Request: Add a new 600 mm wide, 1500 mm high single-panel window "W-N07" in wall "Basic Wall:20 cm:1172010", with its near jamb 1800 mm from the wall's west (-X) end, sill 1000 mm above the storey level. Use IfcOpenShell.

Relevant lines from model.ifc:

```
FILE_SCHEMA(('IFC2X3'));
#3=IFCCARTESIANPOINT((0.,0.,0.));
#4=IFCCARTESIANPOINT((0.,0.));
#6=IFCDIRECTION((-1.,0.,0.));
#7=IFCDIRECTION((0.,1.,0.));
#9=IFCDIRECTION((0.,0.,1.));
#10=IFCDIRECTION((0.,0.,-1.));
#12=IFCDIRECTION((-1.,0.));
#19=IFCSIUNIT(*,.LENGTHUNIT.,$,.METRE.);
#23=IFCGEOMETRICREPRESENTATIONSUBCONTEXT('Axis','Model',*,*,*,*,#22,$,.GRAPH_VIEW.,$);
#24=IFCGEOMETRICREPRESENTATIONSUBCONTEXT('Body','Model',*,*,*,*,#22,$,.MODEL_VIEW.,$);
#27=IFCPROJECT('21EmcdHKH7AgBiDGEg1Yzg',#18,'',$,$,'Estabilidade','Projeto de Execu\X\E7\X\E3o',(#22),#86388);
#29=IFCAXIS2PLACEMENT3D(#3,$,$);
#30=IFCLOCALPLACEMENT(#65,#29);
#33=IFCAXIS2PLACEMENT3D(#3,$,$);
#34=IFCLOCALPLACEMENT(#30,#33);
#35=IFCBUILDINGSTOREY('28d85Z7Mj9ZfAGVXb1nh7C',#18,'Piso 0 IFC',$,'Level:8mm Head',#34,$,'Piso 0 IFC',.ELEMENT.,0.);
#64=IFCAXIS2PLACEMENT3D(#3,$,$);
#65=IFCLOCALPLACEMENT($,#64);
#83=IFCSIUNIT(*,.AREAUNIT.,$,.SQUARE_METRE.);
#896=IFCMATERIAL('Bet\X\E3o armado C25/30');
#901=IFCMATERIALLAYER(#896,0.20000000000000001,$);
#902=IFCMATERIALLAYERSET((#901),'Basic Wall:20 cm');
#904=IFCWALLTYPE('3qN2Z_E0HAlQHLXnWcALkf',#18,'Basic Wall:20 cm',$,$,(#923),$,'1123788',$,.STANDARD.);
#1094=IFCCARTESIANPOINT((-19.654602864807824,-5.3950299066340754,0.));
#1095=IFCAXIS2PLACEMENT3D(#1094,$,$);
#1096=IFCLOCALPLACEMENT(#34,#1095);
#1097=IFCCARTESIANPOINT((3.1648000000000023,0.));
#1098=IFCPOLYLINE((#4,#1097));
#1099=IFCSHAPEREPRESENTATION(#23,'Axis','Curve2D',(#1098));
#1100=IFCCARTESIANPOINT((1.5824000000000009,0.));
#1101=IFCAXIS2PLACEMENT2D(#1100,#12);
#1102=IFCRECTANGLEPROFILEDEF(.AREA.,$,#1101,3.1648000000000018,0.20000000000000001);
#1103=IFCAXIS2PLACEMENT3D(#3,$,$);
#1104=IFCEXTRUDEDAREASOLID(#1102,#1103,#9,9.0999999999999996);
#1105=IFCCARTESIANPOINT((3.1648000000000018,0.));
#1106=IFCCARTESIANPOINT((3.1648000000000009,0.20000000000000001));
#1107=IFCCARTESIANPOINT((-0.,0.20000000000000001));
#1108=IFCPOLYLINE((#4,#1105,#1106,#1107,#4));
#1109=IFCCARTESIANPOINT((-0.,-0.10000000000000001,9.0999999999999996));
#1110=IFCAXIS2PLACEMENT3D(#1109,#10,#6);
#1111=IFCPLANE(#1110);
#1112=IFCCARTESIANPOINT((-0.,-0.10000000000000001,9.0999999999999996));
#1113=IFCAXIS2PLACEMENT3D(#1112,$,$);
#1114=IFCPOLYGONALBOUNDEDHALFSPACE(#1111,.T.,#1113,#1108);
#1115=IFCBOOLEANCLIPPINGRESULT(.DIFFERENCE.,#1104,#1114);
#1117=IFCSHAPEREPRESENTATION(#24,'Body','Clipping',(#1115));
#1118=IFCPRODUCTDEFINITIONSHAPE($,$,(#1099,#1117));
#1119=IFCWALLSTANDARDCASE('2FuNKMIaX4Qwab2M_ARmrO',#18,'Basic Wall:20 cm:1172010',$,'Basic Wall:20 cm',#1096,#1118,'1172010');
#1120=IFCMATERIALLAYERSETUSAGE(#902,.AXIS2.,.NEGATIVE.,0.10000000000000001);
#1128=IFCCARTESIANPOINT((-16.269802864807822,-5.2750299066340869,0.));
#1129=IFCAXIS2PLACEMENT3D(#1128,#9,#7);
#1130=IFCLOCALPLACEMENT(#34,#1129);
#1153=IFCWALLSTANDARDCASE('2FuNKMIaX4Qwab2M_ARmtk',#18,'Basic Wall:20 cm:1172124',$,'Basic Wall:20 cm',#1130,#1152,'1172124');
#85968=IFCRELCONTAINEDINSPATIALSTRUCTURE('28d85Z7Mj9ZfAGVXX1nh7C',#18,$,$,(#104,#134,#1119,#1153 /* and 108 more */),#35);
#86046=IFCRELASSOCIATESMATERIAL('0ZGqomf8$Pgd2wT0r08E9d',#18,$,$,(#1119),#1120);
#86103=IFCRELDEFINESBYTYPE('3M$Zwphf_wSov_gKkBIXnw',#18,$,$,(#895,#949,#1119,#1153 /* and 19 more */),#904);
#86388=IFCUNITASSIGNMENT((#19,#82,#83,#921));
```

```python
import numpy as np
import ifcopenshell
import ifcopenshell.api.feature
import ifcopenshell.api.geometry
import ifcopenshell.api.root
import ifcopenshell.api.spatial
import ifcopenshell.api.type
import ifcopenshell.geom
import ifcopenshell.util.element
import ifcopenshell.util.placement
import ifcopenshell.util.representation
import ifcopenshell.util.shape
import ifcopenshell.util.unit

model = ifcopenshell.open("model.ifc")
unit_scale = ifcopenshell.util.unit.calculate_unit_scale(model)
settings = ifcopenshell.geom.settings()


def volume(element):
    """Net volume in cubic metres, openings subtracted."""
    shape = ifcopenshell.geom.create_shape(settings, element)
    return ifcopenshell.util.shape.get_volume(shape.geometry)


wall = model.by_id(1119)
storey = ifcopenshell.util.element.get_container(wall, ifc_class="IfcBuildingStorey")
context = ifcopenshell.util.representation.get_context(model, "Model", "Body", "MODEL_VIEW")
before = volume(wall)

width, height, from_end, sill = 0.6, 1.5, 1.8, 1  # metres

# The wall runs along its own X axis, and the end named is its -X end.
wall_shape = ifcopenshell.geom.create_shape(settings, wall)
x, y, z = ifcopenshell.util.shape.get_vertices(wall_shape.geometry).T
start = x.min() + from_end
face, thickness = float(y.min()), float(y.max() - y.min())
wall_matrix = ifcopenshell.util.placement.get_local_placement(wall.ObjectPlacement)
level = ifcopenshell.util.placement.get_local_placement(storey.ObjectPlacement)[2, 3]


def in_wall(x, y):
    """Placement at x, y metres in the wall's axes, at sill height."""
    matrix = wall_matrix.copy()
    matrix[:, 3] = wall_matrix @ np.array([x / unit_scale, y / unit_scale, 0.0, 1.0])
    matrix[2, 3] = level + sill / unit_scale
    return matrix


# Opening: a box that overshoots both wall faces by 50 mm.
opening = ifcopenshell.api.root.create_entity(model, ifc_class="IfcOpeningElement")
box = ifcopenshell.api.geometry.add_wall_representation(
    model, context=context, length=width, height=height, thickness=thickness + 0.1
)
ifcopenshell.api.geometry.assign_representation(model, product=opening, representation=box)
ifcopenshell.api.geometry.edit_object_placement(model, product=opening, matrix=in_wall(start, face - 0.05), is_si=False)
ifcopenshell.api.feature.add_feature(model, feature=opening, element=wall)

window = ifcopenshell.api.root.create_entity(model, ifc_class="IfcWindow", name="W-N07")
window.OverallWidth, window.OverallHeight = width / unit_scale, height / unit_scale
body = ifcopenshell.api.geometry.add_window_representation(
    model,
    context=context,
    overall_width=window.OverallWidth,
    overall_height=window.OverallHeight,
    partition_type="SINGLE_PANEL",
)
ifcopenshell.api.geometry.assign_representation(model, product=window, representation=body)
ifcopenshell.api.spatial.assign_container(model, products=[window], relating_structure=storey)
fills = ifcopenshell.api.feature.add_filling(model, opening=opening, element=window)
fills.OwnerHistory = window.OwnerHistory  # required in IFC2X3

# IFC2X3 keeps the operation on the window style.
style = ifcopenshell.api.root.create_entity(model, ifc_class="IfcWindowStyle", name="W-N07")
style.OperationType, style.ConstructionType = "SINGLE_PANEL", "NOTDEFINED"
style.ParameterTakesPrecedence = style.Sizeable = False
ifcopenshell.api.type.assign_type(model, related_objects=[window], relating_type=style)

# Centre the window in the wall's thickness.
ifcopenshell.api.geometry.edit_object_placement(model, product=window, matrix=in_wall(start, face), is_si=False)
window_shape = ifcopenshell.geom.create_shape(settings, window)
depth = ifcopenshell.util.shape.get_vertices(window_shape.geometry)[:, 1]
offset = face + thickness / 2 - (depth.min() + depth.max()) / 2
ifcopenshell.api.geometry.edit_object_placement(model, product=window, matrix=in_wall(start, offset), is_si=False)

after = volume(wall)

print(f"wall volume {before:.3f} -> {after:.3f} m3")

model.write("model-out.ifc")
```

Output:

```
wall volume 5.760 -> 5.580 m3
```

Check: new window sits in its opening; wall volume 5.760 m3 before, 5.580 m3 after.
